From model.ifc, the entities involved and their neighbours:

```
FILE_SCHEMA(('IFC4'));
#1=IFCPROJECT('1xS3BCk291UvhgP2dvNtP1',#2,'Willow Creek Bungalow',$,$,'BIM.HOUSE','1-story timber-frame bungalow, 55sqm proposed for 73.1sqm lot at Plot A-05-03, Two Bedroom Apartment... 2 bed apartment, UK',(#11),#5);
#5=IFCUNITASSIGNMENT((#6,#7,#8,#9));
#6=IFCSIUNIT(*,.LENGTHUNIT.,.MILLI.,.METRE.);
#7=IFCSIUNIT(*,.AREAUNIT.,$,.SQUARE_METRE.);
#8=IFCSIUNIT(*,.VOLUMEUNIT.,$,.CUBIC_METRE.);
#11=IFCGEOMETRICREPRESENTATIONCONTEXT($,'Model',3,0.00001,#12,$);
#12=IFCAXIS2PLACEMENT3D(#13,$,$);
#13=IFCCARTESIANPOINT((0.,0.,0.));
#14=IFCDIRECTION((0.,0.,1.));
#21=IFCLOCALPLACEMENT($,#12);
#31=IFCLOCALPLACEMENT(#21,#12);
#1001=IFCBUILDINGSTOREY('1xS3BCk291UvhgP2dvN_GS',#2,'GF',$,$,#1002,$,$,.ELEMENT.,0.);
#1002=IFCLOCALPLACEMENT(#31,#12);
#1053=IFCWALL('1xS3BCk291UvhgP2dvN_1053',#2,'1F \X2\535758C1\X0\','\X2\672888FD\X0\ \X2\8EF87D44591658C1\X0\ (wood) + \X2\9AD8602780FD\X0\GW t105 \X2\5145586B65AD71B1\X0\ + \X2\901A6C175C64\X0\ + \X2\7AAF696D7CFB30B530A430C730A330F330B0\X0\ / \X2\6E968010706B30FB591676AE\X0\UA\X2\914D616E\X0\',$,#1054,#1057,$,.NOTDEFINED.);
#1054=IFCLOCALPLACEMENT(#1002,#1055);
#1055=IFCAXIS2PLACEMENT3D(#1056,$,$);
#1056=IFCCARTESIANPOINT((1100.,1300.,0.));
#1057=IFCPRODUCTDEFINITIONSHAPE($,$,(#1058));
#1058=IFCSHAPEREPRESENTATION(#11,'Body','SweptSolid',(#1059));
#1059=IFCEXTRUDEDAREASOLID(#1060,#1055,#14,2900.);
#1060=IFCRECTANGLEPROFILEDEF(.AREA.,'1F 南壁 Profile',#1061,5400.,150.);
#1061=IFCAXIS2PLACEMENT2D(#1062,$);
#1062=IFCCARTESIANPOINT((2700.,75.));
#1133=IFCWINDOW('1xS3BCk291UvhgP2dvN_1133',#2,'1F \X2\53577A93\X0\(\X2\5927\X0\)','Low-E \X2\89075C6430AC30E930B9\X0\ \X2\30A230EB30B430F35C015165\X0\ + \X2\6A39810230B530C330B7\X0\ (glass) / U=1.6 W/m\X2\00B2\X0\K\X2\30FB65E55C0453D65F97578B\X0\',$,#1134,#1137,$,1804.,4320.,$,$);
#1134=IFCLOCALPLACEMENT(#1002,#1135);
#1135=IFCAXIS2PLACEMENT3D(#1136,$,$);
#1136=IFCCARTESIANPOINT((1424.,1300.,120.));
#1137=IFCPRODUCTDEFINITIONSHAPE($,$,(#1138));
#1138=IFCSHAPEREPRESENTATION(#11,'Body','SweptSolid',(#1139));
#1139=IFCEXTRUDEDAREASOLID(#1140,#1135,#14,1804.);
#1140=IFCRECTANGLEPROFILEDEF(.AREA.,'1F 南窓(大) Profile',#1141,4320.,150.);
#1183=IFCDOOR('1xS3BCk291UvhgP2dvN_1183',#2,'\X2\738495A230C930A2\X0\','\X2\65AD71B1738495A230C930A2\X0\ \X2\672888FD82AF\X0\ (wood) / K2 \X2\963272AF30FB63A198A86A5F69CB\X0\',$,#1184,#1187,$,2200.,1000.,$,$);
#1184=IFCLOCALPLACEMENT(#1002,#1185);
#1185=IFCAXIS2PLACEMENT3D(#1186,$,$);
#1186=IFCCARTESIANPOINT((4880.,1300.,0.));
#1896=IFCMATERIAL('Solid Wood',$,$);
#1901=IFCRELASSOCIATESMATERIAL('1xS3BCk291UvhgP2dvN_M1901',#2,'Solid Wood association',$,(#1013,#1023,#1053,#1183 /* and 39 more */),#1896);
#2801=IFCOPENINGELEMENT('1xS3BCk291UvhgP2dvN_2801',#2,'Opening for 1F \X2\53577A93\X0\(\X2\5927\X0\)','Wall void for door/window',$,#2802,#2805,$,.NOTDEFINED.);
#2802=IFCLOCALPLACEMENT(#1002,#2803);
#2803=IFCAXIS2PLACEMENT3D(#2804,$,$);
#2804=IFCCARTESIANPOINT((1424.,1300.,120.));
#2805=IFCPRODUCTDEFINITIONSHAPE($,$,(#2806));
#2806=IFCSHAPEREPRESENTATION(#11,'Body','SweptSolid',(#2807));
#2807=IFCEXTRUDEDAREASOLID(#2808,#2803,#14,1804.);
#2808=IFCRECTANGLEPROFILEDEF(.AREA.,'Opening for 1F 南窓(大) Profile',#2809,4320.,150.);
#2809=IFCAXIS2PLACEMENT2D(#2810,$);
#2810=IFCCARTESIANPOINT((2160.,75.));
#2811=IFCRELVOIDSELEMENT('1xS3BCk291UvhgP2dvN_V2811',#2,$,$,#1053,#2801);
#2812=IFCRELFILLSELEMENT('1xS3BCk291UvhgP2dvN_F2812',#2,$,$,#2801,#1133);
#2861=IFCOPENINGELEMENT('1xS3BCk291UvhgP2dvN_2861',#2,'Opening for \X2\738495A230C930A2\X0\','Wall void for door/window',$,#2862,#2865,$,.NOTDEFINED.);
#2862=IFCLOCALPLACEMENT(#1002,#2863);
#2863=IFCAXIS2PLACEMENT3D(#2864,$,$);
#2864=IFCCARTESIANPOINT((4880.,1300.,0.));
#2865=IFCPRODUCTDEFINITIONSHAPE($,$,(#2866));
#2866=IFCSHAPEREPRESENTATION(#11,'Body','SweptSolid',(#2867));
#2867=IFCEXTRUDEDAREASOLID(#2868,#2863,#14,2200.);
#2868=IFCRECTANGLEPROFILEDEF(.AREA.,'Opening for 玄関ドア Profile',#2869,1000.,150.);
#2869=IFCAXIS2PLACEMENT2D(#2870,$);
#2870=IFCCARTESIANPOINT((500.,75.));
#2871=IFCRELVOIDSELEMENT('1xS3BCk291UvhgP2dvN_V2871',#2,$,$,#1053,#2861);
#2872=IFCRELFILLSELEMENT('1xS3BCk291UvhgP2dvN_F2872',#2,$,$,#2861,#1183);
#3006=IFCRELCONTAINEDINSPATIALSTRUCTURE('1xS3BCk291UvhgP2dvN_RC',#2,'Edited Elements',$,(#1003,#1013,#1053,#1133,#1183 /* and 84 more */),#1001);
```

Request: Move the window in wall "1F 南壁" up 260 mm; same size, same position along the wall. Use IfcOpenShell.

```python
import numpy as np
import ifcopenshell
import ifcopenshell.api.geometry
import ifcopenshell.util.placement
import ifcopenshell.util.unit

model = ifcopenshell.open("model.ifc")
unit_scale = ifcopenshell.util.unit.calculate_unit_scale(model)

window = model.by_guid("1xS3BCk291UvhgP2dvN_1133")
opening = window.FillsVoids[0].RelatingOpeningElement
dz = 260.0

shift = np.array([0.0, 0.0, dz])
# The window is not placed relative to its opening, so move both.
for product in (opening, window):
    matrix = ifcopenshell.util.placement.get_local_placement(product.ObjectPlacement)
    matrix[:3, 3] += shift
    ifcopenshell.api.geometry.edit_object_placement(model, product=product, matrix=matrix, is_si=False)

print(f"moved by {dz * unit_scale:+.3f} m")

model.write("model_v2.ifc")
```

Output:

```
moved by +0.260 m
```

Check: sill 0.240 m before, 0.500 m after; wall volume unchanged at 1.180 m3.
